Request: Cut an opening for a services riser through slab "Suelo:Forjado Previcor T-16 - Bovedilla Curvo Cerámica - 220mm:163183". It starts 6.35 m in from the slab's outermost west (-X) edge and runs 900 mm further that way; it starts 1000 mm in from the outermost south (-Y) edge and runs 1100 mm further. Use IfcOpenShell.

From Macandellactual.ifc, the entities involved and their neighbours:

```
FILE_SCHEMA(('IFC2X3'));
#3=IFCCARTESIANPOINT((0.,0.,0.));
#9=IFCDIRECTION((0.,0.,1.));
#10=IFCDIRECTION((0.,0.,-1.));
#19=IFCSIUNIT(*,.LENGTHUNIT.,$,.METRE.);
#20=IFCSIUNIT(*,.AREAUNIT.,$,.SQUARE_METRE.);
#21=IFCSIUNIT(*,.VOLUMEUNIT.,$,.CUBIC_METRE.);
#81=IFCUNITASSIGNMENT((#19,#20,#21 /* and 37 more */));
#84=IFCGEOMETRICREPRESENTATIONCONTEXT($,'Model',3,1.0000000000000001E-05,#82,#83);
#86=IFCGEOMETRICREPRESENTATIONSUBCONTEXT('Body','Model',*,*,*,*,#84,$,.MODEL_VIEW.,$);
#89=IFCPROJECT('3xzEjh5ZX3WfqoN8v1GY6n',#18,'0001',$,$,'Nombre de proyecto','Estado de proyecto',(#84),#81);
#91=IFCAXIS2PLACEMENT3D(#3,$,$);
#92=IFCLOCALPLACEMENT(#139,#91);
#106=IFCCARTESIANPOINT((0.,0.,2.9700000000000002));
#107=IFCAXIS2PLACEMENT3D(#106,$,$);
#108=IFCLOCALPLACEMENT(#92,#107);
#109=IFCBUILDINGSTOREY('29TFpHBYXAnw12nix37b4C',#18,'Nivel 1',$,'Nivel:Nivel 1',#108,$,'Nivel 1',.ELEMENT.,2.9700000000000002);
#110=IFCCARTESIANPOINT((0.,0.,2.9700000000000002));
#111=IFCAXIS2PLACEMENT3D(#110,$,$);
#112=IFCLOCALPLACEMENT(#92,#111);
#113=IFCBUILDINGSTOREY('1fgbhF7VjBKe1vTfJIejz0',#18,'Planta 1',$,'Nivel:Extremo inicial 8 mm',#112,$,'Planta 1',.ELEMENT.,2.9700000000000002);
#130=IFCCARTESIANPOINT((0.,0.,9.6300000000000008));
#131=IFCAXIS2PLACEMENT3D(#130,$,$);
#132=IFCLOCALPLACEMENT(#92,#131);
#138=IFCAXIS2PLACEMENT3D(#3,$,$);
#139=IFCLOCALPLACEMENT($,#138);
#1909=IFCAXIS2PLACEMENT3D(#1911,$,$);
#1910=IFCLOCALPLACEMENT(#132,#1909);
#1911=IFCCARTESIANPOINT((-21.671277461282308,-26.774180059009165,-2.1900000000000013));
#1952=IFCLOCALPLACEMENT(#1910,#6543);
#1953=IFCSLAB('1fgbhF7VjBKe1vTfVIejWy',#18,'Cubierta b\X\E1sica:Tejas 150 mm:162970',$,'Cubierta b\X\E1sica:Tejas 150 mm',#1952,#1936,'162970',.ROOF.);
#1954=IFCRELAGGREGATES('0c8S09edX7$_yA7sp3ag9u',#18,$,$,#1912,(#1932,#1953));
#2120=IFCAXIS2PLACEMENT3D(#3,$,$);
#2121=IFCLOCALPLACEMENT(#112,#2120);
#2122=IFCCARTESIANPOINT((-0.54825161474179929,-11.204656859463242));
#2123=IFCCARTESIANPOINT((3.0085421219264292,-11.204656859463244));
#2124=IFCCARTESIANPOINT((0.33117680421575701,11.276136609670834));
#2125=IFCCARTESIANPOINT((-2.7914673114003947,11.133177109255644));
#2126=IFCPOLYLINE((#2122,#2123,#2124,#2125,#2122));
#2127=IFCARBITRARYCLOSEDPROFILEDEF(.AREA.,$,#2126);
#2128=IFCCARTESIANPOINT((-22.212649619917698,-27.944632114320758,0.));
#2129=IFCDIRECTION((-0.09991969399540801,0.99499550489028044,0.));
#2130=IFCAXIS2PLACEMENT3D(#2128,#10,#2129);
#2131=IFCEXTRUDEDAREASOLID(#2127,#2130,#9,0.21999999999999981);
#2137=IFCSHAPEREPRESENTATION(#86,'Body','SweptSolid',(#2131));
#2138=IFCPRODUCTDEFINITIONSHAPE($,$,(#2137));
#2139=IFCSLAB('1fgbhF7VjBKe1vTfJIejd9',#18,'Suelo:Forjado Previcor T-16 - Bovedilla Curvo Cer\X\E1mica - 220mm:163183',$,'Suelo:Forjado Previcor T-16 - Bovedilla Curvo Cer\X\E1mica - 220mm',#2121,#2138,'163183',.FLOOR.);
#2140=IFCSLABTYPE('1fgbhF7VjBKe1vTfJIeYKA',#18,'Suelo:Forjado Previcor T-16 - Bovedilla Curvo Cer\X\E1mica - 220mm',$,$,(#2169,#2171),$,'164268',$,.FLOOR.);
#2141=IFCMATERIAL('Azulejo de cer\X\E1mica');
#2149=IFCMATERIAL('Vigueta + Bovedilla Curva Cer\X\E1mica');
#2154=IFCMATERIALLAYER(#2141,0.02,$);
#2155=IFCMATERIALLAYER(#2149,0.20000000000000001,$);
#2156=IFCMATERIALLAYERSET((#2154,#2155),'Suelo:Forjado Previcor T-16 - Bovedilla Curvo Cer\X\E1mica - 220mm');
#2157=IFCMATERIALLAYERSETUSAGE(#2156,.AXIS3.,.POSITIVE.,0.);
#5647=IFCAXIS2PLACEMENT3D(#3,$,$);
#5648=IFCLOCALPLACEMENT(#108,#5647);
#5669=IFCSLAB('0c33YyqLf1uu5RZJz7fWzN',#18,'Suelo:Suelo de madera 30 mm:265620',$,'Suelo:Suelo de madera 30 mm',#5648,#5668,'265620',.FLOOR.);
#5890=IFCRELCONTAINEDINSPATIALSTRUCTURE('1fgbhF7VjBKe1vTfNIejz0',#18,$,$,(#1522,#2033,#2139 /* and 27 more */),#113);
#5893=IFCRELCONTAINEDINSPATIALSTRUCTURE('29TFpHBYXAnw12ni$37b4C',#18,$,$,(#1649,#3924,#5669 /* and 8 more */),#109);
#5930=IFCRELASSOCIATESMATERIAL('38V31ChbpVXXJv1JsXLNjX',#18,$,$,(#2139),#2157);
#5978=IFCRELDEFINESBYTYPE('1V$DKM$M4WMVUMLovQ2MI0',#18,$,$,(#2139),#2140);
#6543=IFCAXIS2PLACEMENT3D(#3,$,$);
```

```python
import numpy as np
import ifcopenshell
import ifcopenshell.api.feature
import ifcopenshell.api.geometry
import ifcopenshell.api.root
import ifcopenshell.geom
import ifcopenshell.util.placement
import ifcopenshell.util.representation
import ifcopenshell.util.shape
import ifcopenshell.util.unit

model = ifcopenshell.open("Macandellactual.ifc")
unit_scale = ifcopenshell.util.unit.calculate_unit_scale(model)
settings = ifcopenshell.geom.settings()


def volume(element):
    """Net volume in cubic metres, openings subtracted."""
    shape = ifcopenshell.geom.create_shape(settings, element)
    return ifcopenshell.util.shape.get_volume(shape.geometry)


slab = model.by_guid("1fgbhF7VjBKe1vTfJIejd9")
before = volume(slab)

# Extent in the slab's own axes, in metres. The edges named are its -X and -Y sides.
slab_shape = ifcopenshell.geom.create_shape(settings, slab)
vertices = ifcopenshell.util.shape.get_vertices(slab_shape.geometry)
x_min, y_min, bottom = vertices.min(axis=0)
top = vertices[:, 2].max()

opening = ifcopenshell.api.root.create_entity(model, ifc_class="IfcOpeningElement", name="Services riser opening")
context = ifcopenshell.util.representation.get_context(model, "Model", "Body", "MODEL_VIEW")
width, depth = 0.9, 1.1
outline = [(0.0, 0.0), (width, 0.0), (width, depth), (0.0, depth), (0.0, 0.0)]
# Overshoot both faces by 50 mm so the cut is clean.
shape = ifcopenshell.api.geometry.add_slab_representation(
    model, context=context, depth=top - bottom + 0.1, polyline=outline
)
ifcopenshell.api.geometry.assign_representation(model, product=opening, representation=shape)

matrix = ifcopenshell.util.placement.get_local_placement(slab.ObjectPlacement)
matrix[:, 3] = matrix @ np.append(np.array([x_min + 6.35, y_min + 1, bottom - 0.05]) / unit_scale, 1.0)
ifcopenshell.api.geometry.edit_object_placement(model, product=opening, matrix=matrix, is_si=False)
ifcopenshell.api.feature.add_feature(model, feature=opening, element=slab)

after = volume(slab)

print(f"slab volume {before:.3f} -> {after:.3f} m3")

model.write("Macandellactual_updated.ifc")
```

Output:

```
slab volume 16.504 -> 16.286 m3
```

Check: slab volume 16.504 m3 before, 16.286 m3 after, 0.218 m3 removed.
